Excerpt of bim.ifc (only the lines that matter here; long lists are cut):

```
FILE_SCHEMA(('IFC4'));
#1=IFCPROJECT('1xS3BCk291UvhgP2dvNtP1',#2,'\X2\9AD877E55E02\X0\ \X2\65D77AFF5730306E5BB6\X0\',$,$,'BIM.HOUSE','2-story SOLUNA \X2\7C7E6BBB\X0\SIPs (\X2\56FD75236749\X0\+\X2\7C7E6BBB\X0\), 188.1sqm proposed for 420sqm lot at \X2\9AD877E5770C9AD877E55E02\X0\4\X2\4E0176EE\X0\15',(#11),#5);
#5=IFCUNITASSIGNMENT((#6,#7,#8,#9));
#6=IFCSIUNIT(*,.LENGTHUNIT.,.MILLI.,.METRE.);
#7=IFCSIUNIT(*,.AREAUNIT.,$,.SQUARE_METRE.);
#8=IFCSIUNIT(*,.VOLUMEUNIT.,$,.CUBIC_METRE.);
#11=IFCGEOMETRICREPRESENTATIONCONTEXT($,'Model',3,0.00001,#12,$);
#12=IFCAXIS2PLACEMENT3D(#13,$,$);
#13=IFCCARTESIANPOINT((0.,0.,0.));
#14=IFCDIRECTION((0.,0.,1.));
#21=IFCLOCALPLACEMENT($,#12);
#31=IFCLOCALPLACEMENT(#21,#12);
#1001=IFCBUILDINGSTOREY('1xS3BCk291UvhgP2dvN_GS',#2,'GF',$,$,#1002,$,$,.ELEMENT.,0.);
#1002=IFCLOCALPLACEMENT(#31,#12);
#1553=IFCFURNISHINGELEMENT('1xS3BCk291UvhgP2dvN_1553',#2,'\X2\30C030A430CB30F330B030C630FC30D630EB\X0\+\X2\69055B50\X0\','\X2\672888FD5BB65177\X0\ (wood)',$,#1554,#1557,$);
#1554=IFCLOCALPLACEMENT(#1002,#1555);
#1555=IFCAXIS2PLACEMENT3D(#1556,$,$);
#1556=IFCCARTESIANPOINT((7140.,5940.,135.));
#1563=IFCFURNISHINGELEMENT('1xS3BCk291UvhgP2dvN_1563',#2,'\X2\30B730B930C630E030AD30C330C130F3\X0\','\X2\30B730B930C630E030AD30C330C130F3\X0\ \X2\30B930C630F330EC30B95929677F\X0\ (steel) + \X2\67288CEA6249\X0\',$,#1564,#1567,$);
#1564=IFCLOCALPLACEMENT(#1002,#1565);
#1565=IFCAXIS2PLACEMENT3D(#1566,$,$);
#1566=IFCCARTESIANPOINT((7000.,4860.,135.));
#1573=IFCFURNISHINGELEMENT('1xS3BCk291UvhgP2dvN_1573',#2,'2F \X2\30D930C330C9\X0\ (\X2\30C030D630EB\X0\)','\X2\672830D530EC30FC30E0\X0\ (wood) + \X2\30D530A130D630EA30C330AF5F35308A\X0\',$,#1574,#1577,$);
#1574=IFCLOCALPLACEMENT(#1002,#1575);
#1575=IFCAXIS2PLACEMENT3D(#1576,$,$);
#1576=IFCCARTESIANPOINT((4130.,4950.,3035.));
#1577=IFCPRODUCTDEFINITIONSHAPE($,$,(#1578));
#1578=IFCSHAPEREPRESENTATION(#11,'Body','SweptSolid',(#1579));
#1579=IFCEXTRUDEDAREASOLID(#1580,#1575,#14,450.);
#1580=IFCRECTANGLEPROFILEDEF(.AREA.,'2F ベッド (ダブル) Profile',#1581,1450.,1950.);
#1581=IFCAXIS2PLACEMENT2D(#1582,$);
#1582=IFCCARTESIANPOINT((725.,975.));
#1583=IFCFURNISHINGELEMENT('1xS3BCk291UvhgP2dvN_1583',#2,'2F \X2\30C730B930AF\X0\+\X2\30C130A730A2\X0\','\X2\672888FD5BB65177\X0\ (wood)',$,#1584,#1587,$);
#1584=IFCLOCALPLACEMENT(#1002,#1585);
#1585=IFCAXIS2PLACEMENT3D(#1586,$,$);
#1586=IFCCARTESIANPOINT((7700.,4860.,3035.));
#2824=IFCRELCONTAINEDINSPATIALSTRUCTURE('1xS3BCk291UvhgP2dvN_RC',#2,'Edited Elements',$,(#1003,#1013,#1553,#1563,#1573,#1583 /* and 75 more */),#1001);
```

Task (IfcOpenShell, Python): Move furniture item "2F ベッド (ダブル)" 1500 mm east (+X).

```python
import ifcopenshell
import ifcopenshell.api.geometry
import ifcopenshell.util.placement
import ifcopenshell.util.unit

model = ifcopenshell.open("bim.ifc")
unit_scale = ifcopenshell.util.unit.calculate_unit_scale(model)

item = model.by_guid("1xS3BCk291UvhgP2dvN_1573")
matrix = ifcopenshell.util.placement.get_local_placement(item.ObjectPlacement)
matrix[0, 3] += 1.5 / unit_scale
ifcopenshell.api.geometry.edit_object_placement(model, product=item, matrix=matrix, is_si=False)

print(ifcopenshell.util.placement.get_local_placement(item.ObjectPlacement).round(3) + 0.0)

model.write("bim-out.ifc")
```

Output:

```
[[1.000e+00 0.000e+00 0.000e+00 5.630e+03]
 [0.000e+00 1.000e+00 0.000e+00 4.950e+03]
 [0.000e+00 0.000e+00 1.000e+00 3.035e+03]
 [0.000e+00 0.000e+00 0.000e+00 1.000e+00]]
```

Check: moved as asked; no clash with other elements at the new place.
